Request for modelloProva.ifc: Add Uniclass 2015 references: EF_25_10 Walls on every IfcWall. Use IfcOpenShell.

First a look at what the model holds.

```python
import ifcopenshell

model = ifcopenshell.open("modelloProva.ifc")
print(model.schema)
print("classifications:", [c.Name for c in model.by_type("IfcClassification")])
for ifc_class in ("IfcDoor", "IfcRoof", "IfcStair", "IfcWall", "IfcWindow"):
    print(ifc_class, len(model.by_type(ifc_class)))
```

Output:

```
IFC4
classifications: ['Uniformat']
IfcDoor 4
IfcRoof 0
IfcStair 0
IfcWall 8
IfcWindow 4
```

```python
import ifcopenshell
import ifcopenshell.api.classification

model = ifcopenshell.open("modelloProva.ifc")

system = ifcopenshell.api.classification.add_classification(model, classification="Uniclass 2015")

codes = {
    "IfcWall": ("EF_25_10", "Walls"),
}
for ifc_class, (code, name) in codes.items():
    products = model.by_type(ifc_class)
    ifcopenshell.api.classification.add_reference(
        model, products=products, classification=system, identification=code, name=name
    )
    print(code, len(products))

model.write("modelloProva_updated.ifc")
```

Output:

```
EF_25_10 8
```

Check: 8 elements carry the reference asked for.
